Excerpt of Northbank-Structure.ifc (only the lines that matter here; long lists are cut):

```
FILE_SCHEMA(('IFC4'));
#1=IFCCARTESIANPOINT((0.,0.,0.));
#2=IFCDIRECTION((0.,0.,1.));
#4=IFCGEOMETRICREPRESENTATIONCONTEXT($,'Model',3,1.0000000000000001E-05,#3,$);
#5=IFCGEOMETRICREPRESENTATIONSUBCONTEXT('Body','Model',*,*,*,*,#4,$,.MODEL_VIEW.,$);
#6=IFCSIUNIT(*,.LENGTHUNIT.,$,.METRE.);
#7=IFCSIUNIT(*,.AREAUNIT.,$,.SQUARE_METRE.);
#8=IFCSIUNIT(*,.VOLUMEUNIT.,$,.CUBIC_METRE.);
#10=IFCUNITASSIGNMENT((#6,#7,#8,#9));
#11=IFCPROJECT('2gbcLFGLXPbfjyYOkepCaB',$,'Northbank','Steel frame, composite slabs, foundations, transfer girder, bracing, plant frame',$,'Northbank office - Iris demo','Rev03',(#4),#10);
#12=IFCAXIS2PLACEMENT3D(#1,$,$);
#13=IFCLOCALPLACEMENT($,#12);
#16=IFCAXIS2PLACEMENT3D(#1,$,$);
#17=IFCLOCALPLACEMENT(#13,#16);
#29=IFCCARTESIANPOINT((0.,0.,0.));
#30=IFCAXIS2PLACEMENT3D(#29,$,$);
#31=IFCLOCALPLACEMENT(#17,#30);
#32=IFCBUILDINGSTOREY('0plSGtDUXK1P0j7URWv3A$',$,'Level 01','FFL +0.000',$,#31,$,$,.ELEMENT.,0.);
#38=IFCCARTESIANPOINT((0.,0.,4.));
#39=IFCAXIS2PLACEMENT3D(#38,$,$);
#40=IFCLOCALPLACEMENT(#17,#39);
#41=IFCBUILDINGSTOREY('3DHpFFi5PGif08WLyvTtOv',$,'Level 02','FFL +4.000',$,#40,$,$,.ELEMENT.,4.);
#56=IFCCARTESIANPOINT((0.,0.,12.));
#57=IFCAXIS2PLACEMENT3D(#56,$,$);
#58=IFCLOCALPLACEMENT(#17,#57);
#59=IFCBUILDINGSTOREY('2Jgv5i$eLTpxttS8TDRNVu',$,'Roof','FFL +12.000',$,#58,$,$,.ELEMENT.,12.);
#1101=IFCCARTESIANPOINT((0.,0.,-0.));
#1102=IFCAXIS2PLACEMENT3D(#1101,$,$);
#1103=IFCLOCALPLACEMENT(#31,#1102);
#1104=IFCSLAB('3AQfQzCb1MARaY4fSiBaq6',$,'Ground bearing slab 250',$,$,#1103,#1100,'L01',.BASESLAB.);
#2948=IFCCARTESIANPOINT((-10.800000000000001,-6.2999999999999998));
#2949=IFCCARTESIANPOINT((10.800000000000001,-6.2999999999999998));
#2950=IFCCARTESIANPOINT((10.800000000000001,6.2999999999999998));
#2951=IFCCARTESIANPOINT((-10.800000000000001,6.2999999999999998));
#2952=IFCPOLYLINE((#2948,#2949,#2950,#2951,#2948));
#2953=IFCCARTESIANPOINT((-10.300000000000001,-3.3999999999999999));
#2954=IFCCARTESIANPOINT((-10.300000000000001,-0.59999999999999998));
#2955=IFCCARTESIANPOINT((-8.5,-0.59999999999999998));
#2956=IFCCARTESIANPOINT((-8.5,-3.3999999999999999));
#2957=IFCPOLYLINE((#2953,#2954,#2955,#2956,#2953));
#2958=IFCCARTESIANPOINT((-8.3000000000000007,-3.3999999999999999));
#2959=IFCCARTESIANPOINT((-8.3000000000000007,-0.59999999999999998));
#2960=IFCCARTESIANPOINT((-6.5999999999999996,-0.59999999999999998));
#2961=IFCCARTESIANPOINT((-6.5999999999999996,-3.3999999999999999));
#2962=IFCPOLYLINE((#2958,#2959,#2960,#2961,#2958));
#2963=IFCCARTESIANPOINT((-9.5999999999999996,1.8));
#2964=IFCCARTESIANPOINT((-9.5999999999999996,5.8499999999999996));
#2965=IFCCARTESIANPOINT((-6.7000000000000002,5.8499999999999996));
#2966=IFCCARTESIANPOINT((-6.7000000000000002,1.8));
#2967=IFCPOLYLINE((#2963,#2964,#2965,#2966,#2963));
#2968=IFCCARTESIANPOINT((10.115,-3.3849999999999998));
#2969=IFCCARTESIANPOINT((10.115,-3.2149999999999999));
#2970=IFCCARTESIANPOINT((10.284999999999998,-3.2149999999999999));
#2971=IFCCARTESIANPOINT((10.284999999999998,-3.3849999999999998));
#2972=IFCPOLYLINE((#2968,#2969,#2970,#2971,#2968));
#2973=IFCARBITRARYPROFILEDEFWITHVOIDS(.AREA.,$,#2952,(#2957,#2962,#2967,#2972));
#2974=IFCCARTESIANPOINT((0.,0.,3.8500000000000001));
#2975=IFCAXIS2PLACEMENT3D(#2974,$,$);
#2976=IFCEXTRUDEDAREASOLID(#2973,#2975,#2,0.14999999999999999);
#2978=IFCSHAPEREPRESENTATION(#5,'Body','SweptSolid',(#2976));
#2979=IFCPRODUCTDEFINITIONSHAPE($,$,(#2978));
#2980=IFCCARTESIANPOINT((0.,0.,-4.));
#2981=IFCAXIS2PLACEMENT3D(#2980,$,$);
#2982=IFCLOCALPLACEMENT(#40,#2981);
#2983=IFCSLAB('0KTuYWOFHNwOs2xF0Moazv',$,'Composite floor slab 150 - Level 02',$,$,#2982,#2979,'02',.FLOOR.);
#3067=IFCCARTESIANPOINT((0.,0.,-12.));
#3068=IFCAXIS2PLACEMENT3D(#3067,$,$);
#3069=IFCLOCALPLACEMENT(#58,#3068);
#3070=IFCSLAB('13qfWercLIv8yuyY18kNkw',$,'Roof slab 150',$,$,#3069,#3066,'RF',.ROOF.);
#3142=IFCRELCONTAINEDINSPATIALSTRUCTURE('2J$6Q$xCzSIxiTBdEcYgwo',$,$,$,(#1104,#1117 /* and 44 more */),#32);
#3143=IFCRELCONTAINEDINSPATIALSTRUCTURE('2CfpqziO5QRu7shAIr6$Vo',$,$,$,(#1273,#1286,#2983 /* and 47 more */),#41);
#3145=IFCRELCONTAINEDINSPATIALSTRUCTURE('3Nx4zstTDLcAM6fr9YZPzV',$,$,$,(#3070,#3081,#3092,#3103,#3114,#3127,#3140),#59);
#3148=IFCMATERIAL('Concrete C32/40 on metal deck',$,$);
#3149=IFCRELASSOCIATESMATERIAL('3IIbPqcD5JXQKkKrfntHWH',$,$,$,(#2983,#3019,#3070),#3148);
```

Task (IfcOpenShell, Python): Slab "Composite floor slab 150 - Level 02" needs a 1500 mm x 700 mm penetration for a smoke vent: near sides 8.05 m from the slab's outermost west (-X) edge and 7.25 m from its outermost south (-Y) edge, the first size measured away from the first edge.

```python
import numpy as np
import ifcopenshell
import ifcopenshell.api.feature
import ifcopenshell.api.geometry
import ifcopenshell.api.root
import ifcopenshell.geom
import ifcopenshell.util.placement
import ifcopenshell.util.representation
import ifcopenshell.util.shape
import ifcopenshell.util.unit

model = ifcopenshell.open("Northbank-Structure.ifc")
unit_scale = ifcopenshell.util.unit.calculate_unit_scale(model)
settings = ifcopenshell.geom.settings()


def volume(element):
    """Net volume in cubic metres, openings subtracted."""
    shape = ifcopenshell.geom.create_shape(settings, element)
    return ifcopenshell.util.shape.get_volume(shape.geometry)


slab = model.by_guid("0KTuYWOFHNwOs2xF0Moazv")
before = volume(slab)

# Extent in the slab's own axes, in metres. The edges named are its -X and -Y sides.
slab_shape = ifcopenshell.geom.create_shape(settings, slab)
vertices = ifcopenshell.util.shape.get_vertices(slab_shape.geometry)
x_min, y_min, bottom = vertices.min(axis=0)
top = vertices[:, 2].max()

opening = ifcopenshell.api.root.create_entity(model, ifc_class="IfcOpeningElement", name="Smoke vent opening", predefined_type="OPENING")
context = ifcopenshell.util.representation.get_context(model, "Model", "Body", "MODEL_VIEW")
width, depth = 1.5, 0.7
outline = [(0.0, 0.0), (width, 0.0), (width, depth), (0.0, depth), (0.0, 0.0)]
# Overshoot both faces by 50 mm so the cut is clean.
shape = ifcopenshell.api.geometry.add_slab_representation(
    model, context=context, depth=top - bottom + 0.1, polyline=outline
)
ifcopenshell.api.geometry.assign_representation(model, product=opening, representation=shape)

matrix = ifcopenshell.util.placement.get_local_placement(slab.ObjectPlacement)
matrix[:, 3] = matrix @ np.append(np.array([x_min + 8.05, y_min + 7.25, bottom - 0.05]) / unit_scale, 1.0)
ifcopenshell.api.geometry.edit_object_placement(model, product=opening, matrix=matrix, is_si=False)
ifcopenshell.api.feature.add_feature(model, feature=opening, element=slab)

after = volume(slab)

print(f"slab volume {before:.3f} -> {after:.3f} m3")

model.write("Northbank-Structure_edited.ifc")
```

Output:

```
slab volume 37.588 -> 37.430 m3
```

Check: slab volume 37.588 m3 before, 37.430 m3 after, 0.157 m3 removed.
